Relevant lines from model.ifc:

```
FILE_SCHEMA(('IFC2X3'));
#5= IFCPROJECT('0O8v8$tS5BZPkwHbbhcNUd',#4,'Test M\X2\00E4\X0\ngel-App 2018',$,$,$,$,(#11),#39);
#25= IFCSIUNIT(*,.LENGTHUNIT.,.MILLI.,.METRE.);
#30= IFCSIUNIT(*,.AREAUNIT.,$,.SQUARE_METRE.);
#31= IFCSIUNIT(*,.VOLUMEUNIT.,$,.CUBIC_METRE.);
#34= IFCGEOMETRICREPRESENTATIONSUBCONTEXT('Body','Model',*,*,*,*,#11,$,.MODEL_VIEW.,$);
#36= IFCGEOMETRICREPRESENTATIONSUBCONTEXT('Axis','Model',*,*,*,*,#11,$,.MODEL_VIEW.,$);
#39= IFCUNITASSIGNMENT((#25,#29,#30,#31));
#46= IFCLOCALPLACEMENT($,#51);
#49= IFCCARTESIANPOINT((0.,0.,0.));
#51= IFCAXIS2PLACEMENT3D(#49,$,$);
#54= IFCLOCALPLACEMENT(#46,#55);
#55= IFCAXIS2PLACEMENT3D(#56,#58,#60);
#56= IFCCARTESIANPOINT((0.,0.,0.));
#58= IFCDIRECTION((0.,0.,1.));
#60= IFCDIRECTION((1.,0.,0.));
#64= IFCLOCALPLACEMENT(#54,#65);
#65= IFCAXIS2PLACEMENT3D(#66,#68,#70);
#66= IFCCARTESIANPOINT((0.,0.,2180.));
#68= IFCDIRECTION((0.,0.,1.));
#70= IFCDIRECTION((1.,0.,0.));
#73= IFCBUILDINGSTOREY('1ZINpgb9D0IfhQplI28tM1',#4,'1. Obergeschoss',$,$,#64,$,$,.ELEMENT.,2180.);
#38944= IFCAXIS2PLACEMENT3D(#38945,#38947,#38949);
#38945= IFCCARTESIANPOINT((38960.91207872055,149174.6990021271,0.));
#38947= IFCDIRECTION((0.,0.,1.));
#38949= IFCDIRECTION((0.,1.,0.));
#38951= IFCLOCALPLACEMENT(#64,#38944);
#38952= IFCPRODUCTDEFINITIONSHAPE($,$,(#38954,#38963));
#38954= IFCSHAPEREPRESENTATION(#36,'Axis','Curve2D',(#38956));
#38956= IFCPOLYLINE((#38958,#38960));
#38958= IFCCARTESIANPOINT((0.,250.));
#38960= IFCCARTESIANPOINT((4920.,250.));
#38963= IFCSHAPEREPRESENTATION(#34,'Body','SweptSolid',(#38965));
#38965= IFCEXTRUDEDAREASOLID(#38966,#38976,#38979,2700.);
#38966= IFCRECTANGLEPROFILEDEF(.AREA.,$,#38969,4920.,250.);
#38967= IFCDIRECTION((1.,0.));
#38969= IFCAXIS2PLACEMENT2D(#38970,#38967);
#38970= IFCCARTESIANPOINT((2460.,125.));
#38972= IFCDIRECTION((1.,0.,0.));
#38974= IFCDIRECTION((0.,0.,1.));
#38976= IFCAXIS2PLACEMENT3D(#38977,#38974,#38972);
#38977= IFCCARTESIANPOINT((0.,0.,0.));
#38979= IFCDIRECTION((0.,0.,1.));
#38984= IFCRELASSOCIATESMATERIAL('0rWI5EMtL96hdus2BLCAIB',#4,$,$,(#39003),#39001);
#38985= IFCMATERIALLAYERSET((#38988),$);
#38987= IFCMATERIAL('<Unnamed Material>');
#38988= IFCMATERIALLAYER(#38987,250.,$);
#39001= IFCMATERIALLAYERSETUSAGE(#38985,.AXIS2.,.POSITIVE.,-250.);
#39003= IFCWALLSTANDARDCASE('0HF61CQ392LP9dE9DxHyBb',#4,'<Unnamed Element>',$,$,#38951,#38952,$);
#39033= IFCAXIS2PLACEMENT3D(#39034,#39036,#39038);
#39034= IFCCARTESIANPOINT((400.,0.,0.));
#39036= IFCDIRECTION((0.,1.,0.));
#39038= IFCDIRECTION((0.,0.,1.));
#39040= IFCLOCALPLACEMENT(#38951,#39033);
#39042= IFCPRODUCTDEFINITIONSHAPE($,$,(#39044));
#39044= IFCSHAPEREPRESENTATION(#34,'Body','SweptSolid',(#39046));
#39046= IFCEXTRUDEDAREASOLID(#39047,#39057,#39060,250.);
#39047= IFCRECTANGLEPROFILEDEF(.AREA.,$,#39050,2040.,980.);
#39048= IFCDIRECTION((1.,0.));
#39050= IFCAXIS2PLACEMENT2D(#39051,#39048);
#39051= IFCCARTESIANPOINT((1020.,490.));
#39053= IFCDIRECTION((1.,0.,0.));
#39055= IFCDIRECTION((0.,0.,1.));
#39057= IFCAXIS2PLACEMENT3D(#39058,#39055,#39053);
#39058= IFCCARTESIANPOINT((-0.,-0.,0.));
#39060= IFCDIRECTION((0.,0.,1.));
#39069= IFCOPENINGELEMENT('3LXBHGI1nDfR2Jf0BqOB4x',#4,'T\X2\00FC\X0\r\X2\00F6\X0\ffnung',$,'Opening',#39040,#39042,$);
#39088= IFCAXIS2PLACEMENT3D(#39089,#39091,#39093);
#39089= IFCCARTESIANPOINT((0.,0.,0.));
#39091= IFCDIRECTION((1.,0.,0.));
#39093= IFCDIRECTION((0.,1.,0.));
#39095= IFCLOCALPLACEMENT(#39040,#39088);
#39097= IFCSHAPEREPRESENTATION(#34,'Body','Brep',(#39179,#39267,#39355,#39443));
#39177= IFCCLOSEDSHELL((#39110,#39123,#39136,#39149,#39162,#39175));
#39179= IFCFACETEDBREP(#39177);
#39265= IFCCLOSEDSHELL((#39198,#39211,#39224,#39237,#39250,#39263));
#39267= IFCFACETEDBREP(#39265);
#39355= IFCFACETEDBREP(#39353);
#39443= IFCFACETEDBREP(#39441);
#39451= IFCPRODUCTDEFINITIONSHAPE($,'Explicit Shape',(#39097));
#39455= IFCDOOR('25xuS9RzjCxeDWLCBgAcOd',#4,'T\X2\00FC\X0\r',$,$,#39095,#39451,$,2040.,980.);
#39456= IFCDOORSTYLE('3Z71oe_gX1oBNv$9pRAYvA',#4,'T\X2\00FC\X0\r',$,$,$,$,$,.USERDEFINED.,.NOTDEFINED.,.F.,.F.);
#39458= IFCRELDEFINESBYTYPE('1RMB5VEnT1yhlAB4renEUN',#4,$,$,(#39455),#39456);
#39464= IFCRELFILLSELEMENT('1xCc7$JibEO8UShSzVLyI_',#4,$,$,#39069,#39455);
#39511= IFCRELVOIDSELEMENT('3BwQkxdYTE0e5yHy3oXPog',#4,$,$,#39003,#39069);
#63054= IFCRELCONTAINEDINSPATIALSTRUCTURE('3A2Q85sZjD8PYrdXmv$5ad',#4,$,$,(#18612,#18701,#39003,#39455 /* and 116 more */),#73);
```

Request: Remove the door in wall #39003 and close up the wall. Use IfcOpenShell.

```python
import ifcopenshell
import ifcopenshell.api.feature
import ifcopenshell.api.root
import ifcopenshell.geom
import ifcopenshell.util.shape

model = ifcopenshell.open("model.ifc")
settings = ifcopenshell.geom.settings()


def volume(element):
    """Net volume in cubic metres, openings subtracted."""
    shape = ifcopenshell.geom.create_shape(settings, element)
    return ifcopenshell.util.shape.get_volume(shape.geometry)


door = model.by_guid("25xuS9RzjCxeDWLCBgAcOd")
opening = door.FillsVoids[0].RelatingOpeningElement
wall = opening.VoidsElements[0].RelatingBuildingElement
before = volume(wall)

ifcopenshell.api.root.remove_product(model, product=door)
ifcopenshell.api.feature.remove_feature(model, feature=opening)

after = volume(wall)

print(f"wall volume {before:.3f} -> {after:.3f} m3")

model.write("model_rev.ifc")
```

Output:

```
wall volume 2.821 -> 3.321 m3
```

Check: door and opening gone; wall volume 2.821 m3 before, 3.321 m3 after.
